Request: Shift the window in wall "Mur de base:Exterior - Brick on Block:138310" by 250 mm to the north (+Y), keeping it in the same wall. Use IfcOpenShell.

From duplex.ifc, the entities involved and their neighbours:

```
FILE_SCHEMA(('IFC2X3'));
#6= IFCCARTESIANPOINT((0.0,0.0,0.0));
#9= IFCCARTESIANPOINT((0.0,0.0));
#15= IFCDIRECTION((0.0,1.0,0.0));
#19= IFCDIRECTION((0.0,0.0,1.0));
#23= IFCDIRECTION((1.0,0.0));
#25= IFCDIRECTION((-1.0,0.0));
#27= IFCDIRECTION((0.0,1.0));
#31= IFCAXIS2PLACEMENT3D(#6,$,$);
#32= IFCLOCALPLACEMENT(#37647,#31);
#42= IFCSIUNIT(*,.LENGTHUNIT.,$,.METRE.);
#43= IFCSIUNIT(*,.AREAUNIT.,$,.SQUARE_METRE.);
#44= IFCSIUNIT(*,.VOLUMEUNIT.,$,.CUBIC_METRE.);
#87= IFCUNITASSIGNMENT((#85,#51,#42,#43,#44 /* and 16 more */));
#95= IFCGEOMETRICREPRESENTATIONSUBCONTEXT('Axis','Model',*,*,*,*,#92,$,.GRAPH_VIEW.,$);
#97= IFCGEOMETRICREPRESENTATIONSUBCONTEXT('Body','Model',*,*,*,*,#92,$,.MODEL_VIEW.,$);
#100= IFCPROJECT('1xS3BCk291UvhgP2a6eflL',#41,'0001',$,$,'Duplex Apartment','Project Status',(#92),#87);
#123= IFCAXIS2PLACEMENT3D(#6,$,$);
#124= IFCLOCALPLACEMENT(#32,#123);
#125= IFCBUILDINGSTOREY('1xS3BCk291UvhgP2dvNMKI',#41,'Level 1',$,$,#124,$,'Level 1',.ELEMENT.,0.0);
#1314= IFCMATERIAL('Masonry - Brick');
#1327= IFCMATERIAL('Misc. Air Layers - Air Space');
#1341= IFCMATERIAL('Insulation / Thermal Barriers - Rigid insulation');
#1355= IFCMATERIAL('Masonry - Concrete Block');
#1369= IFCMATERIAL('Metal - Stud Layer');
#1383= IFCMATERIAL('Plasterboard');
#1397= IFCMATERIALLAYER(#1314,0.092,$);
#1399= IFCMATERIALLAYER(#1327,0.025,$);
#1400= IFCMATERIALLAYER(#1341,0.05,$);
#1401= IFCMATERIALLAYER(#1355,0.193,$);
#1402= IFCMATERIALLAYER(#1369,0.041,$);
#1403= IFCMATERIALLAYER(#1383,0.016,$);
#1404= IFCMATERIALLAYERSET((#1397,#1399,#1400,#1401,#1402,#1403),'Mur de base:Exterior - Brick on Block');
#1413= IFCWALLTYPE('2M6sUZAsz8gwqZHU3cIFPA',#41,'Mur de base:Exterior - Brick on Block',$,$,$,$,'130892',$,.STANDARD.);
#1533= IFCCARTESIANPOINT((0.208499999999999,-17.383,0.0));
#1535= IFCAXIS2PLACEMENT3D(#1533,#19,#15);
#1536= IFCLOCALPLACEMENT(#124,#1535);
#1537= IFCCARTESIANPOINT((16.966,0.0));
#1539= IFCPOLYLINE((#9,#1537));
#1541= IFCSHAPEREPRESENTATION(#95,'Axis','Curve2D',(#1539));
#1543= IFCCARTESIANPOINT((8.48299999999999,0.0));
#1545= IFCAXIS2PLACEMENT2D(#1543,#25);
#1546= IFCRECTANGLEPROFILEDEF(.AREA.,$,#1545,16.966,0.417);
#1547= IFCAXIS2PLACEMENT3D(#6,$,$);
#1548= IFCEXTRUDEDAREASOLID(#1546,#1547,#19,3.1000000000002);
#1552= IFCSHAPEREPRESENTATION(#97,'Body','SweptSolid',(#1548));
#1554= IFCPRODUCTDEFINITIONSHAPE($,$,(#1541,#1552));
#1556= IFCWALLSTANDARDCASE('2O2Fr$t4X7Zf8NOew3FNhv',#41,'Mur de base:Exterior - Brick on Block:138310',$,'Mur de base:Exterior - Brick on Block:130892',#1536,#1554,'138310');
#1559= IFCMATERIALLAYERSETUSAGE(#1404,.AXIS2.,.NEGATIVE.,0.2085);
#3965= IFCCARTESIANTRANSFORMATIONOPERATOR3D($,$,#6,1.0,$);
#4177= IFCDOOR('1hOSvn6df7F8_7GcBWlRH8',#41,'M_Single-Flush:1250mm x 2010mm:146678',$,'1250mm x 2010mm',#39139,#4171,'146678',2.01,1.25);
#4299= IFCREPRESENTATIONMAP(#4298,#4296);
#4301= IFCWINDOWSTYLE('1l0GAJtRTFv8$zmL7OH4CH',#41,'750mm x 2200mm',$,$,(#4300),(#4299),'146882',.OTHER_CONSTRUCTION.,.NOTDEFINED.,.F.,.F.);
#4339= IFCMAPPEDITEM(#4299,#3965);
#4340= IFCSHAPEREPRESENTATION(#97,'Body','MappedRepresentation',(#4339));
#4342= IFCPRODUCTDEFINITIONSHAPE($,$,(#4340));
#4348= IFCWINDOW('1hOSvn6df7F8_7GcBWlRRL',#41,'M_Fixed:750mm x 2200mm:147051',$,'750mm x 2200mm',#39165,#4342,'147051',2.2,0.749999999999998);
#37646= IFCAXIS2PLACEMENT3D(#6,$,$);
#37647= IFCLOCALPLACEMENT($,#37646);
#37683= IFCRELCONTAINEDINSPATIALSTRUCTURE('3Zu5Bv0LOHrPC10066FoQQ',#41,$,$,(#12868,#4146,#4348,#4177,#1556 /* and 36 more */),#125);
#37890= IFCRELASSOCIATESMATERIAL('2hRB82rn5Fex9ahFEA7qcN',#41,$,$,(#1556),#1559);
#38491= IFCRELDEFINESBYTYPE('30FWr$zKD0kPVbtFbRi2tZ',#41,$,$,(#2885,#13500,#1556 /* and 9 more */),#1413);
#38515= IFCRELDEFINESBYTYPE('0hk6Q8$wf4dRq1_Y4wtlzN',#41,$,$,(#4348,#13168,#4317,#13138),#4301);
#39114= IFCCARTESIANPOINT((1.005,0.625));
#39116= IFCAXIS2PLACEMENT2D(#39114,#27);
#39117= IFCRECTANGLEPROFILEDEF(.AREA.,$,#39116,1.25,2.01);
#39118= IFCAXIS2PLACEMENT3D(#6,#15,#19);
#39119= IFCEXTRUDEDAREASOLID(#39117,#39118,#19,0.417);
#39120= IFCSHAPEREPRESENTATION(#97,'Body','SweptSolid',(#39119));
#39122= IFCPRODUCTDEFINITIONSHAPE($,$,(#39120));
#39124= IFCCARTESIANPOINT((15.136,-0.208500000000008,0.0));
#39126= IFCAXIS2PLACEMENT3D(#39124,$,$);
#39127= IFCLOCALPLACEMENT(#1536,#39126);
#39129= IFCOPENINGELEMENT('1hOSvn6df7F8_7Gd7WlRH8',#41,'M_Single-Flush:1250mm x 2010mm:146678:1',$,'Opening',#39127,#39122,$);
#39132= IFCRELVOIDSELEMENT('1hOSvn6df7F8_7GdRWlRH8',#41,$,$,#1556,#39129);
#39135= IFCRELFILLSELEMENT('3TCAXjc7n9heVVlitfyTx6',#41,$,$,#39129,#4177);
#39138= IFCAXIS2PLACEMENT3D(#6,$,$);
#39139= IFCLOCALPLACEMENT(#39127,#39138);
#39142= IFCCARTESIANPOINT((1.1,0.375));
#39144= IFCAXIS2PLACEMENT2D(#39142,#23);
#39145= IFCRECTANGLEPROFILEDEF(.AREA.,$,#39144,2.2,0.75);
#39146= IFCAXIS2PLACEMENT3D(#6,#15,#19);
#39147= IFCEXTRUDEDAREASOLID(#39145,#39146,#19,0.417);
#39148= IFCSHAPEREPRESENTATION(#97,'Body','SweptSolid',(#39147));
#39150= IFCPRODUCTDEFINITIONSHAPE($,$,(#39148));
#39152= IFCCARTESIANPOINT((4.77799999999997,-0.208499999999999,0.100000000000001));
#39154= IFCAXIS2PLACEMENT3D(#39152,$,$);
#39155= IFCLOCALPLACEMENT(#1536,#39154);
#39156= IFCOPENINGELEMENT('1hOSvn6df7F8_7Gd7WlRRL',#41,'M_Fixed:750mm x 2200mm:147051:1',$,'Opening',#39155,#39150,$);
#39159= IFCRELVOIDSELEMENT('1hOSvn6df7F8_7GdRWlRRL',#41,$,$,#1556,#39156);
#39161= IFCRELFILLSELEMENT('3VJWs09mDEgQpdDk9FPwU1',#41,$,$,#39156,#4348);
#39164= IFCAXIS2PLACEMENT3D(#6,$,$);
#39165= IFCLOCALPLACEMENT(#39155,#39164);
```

```python
import ifcopenshell
import ifcopenshell.api.geometry
import ifcopenshell.util.placement
import ifcopenshell.util.unit

model = ifcopenshell.open("duplex.ifc")
unit_scale = ifcopenshell.util.unit.calculate_unit_scale(model)

window = model.by_guid("1hOSvn6df7F8_7GcBWlRRL")
opening = window.FillsVoids[0].RelatingOpeningElement
wall = opening.VoidsElements[0].RelatingBuildingElement

wall_matrix = ifcopenshell.util.placement.get_local_placement(wall.ObjectPlacement)
shift = wall_matrix[:3, 0] * 0.25 / unit_scale
before = ifcopenshell.util.placement.get_local_placement(window.ObjectPlacement)[:3, 3].copy()

# The window is placed relative to its opening, so it follows when the opening moves.
matrix = ifcopenshell.util.placement.get_local_placement(opening.ObjectPlacement)
matrix[:3, 3] += shift
ifcopenshell.api.geometry.edit_object_placement(
    model, product=opening, matrix=matrix, is_si=False, should_transform_children=True
)

after = ifcopenshell.util.placement.get_local_placement(window.ObjectPlacement)[:3, 3]
print("window moved by", (after - before).round(3) + 0.0)

model.write("duplex_rev.ifc")
```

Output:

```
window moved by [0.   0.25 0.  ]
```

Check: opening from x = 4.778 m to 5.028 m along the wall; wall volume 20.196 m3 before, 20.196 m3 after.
